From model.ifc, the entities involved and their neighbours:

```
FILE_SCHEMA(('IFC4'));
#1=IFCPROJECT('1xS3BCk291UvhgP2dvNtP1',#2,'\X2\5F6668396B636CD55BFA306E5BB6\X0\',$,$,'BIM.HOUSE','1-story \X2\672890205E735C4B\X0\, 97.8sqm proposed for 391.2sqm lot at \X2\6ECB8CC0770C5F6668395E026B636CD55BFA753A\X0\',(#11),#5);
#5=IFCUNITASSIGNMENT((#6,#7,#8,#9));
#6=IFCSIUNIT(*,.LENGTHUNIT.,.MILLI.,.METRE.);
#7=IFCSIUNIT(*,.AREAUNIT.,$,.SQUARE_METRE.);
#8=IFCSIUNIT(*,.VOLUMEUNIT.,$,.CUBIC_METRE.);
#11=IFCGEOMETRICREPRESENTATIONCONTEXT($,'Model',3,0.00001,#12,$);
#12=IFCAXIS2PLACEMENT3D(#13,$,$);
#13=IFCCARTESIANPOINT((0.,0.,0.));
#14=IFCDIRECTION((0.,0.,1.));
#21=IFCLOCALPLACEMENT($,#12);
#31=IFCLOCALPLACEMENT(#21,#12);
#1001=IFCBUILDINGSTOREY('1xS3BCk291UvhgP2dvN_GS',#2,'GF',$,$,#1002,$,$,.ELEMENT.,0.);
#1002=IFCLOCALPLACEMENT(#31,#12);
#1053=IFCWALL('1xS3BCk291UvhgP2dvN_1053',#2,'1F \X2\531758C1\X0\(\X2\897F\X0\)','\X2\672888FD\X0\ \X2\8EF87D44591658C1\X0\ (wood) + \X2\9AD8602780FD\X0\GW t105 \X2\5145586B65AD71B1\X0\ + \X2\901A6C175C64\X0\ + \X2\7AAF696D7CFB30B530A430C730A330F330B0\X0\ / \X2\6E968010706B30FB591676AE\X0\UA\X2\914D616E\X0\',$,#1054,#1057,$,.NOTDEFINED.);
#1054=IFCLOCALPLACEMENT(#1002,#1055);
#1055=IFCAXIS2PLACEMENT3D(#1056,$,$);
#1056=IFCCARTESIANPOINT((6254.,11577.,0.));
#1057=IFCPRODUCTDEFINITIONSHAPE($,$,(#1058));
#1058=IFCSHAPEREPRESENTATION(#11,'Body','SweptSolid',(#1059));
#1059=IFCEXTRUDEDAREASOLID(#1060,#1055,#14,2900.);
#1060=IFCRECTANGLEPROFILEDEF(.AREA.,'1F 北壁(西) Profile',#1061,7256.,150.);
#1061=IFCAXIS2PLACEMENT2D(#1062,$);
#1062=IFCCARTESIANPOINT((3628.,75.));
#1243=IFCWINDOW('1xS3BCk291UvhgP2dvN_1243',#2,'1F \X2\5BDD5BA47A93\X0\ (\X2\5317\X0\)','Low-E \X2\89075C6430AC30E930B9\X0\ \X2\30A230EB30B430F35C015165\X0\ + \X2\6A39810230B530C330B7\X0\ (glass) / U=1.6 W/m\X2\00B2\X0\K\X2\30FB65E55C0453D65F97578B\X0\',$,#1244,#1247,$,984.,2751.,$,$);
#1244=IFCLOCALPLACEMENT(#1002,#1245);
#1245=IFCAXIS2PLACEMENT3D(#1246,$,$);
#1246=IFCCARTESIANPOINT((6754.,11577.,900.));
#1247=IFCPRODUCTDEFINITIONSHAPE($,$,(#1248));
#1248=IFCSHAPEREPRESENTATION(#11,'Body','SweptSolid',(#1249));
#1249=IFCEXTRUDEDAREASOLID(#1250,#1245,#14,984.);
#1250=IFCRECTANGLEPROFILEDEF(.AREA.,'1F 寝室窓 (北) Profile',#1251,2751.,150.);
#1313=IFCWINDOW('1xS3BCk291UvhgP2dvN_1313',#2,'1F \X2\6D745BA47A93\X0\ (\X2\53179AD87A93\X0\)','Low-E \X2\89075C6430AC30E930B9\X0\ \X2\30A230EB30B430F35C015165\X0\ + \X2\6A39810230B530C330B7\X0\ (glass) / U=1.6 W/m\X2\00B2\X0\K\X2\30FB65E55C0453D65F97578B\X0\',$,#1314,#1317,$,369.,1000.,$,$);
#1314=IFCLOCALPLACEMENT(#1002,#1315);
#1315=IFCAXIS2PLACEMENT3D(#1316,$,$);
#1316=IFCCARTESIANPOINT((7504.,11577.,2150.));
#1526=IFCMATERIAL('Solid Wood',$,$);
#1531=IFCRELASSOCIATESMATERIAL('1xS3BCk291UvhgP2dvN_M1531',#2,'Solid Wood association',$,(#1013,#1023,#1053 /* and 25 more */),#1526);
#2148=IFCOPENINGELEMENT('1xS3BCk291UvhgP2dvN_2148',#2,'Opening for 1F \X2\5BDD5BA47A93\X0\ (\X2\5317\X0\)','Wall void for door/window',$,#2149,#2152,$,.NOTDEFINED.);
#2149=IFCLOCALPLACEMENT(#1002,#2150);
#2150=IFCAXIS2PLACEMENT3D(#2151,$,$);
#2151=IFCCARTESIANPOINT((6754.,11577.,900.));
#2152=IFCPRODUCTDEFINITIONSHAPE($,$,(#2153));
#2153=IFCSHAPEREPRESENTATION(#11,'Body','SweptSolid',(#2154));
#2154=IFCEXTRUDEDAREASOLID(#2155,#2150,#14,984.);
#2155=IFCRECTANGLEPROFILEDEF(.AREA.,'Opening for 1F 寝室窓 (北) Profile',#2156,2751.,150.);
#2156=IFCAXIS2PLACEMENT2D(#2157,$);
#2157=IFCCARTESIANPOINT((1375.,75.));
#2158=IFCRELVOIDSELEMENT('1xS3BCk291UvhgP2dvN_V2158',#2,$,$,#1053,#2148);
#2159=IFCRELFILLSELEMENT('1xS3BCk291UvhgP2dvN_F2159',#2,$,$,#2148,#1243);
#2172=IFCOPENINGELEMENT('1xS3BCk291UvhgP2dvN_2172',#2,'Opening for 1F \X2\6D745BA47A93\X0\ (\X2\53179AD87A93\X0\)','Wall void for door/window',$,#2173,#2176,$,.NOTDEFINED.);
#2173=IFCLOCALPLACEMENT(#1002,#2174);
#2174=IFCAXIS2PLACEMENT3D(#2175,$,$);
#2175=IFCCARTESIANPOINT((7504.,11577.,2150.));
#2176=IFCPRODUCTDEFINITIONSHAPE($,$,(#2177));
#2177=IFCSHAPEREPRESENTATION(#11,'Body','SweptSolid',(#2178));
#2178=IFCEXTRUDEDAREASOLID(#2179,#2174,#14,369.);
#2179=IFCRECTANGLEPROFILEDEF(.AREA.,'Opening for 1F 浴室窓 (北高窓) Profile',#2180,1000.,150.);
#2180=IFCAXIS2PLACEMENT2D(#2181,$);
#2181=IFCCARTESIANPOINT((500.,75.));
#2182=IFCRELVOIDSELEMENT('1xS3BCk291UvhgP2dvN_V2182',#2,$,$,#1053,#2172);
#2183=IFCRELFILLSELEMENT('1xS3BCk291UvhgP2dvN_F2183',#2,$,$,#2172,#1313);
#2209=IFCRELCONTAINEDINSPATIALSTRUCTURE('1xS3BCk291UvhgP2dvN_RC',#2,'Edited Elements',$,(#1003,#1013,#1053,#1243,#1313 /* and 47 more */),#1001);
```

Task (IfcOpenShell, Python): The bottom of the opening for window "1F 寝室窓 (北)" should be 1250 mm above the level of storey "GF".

```python
import numpy as np
import ifcopenshell
import ifcopenshell.api.geometry
import ifcopenshell.geom
import ifcopenshell.util.element
import ifcopenshell.util.placement
import ifcopenshell.util.shape
import ifcopenshell.util.unit

model = ifcopenshell.open("model.ifc")
unit_scale = ifcopenshell.util.unit.calculate_unit_scale(model)

window = model.by_id(1243)
opening = window.FillsVoids[0].RelatingOpeningElement
storey = ifcopenshell.util.element.get_container(window, ifc_class="IfcBuildingStorey")
level = ifcopenshell.util.placement.get_local_placement(storey.ObjectPlacement)[2, 3]

# The opening's origin need not be at the sill, so measure its lowest point.
shape = ifcopenshell.geom.create_shape(ifcopenshell.geom.settings(), opening)
bottom = ifcopenshell.util.shape.get_shape_bottom_elevation(shape, shape.geometry) / unit_scale
dz = level + 1250.0 - bottom

shift = np.array([0.0, 0.0, dz])
# The window is not placed relative to its opening, so move both.
for product in (opening, window):
    matrix = ifcopenshell.util.placement.get_local_placement(product.ObjectPlacement)
    matrix[:3, 3] += shift
    ifcopenshell.api.geometry.edit_object_placement(model, product=product, matrix=matrix, is_si=False)

print(f"moved by {dz * unit_scale:+.3f} m")

model.write("model_rev.ifc")
```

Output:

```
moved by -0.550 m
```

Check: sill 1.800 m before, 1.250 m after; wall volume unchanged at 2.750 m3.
